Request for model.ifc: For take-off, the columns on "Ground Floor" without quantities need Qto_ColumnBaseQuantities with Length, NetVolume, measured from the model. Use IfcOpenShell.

First a look at what the model holds.

```python
import ifcopenshell
import ifcopenshell.util.element
import ifcopenshell.util.unit

model = ifcopenshell.open("model.ifc")
print(model.schema)
for unit_type in ("LENGTHUNIT", "AREAUNIT", "VOLUMEUNIT"):
    print(unit_type, ifcopenshell.util.unit.calculate_unit_scale(model, unit_type))
storey = next(s for s in model.by_type("IfcBuildingStorey") if s.Name == "Ground Floor")
columns = [e for e in ifcopenshell.util.element.get_decomposition(storey) if e.is_a("IfcColumn")]
for e in sorted(columns, key=lambda e: e.id()):
    print(e.id(), e.is_a(), e.Name, list(ifcopenshell.util.element.get_psets(e, qtos_only=True)), sep=" | ")
```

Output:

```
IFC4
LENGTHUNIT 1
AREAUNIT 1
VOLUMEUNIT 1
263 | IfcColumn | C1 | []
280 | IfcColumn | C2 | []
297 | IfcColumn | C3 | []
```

```python
import ifcopenshell
import ifcopenshell.api.pset
import ifcopenshell.geom
import ifcopenshell.util.element
import ifcopenshell.util.shape
import ifcopenshell.util.unit

model = ifcopenshell.open("model.ifc")
unit_scale = ifcopenshell.util.unit.calculate_unit_scale(model)
volume_scale = ifcopenshell.util.unit.calculate_unit_scale(model, "VOLUMEUNIT")
settings = ifcopenshell.geom.settings()

storey = next(s for s in model.by_type("IfcBuildingStorey") if s.Name == "Ground Floor")
columns = [e for e in ifcopenshell.util.element.get_decomposition(storey) if e.is_a("IfcColumn")]

for e in sorted(columns, key=lambda e: e.id()):
    if ifcopenshell.util.element.get_psets(e, qtos_only=True, should_inherit=False):
        continue
    # Geometry comes back in metres, in the element's own axes.
    shape = ifcopenshell.geom.create_shape(settings, e)
    values = {
        "Length": ifcopenshell.util.shape.get_z(shape.geometry) / unit_scale,
        "NetVolume": ifcopenshell.util.shape.get_volume(shape.geometry) / volume_scale,
    }
    qto = ifcopenshell.api.pset.add_qto(model, product=e, name="Qto_ColumnBaseQuantities")
    ifcopenshell.api.pset.edit_qto(model, qto=qto, properties=values)
    print(e.id(), {k: round(v, 3) for k, v in values.items()})

model.write("model_rev.ifc")
```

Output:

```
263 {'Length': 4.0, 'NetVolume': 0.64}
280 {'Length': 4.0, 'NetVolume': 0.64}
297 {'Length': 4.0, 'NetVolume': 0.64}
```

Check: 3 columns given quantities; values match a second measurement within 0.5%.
